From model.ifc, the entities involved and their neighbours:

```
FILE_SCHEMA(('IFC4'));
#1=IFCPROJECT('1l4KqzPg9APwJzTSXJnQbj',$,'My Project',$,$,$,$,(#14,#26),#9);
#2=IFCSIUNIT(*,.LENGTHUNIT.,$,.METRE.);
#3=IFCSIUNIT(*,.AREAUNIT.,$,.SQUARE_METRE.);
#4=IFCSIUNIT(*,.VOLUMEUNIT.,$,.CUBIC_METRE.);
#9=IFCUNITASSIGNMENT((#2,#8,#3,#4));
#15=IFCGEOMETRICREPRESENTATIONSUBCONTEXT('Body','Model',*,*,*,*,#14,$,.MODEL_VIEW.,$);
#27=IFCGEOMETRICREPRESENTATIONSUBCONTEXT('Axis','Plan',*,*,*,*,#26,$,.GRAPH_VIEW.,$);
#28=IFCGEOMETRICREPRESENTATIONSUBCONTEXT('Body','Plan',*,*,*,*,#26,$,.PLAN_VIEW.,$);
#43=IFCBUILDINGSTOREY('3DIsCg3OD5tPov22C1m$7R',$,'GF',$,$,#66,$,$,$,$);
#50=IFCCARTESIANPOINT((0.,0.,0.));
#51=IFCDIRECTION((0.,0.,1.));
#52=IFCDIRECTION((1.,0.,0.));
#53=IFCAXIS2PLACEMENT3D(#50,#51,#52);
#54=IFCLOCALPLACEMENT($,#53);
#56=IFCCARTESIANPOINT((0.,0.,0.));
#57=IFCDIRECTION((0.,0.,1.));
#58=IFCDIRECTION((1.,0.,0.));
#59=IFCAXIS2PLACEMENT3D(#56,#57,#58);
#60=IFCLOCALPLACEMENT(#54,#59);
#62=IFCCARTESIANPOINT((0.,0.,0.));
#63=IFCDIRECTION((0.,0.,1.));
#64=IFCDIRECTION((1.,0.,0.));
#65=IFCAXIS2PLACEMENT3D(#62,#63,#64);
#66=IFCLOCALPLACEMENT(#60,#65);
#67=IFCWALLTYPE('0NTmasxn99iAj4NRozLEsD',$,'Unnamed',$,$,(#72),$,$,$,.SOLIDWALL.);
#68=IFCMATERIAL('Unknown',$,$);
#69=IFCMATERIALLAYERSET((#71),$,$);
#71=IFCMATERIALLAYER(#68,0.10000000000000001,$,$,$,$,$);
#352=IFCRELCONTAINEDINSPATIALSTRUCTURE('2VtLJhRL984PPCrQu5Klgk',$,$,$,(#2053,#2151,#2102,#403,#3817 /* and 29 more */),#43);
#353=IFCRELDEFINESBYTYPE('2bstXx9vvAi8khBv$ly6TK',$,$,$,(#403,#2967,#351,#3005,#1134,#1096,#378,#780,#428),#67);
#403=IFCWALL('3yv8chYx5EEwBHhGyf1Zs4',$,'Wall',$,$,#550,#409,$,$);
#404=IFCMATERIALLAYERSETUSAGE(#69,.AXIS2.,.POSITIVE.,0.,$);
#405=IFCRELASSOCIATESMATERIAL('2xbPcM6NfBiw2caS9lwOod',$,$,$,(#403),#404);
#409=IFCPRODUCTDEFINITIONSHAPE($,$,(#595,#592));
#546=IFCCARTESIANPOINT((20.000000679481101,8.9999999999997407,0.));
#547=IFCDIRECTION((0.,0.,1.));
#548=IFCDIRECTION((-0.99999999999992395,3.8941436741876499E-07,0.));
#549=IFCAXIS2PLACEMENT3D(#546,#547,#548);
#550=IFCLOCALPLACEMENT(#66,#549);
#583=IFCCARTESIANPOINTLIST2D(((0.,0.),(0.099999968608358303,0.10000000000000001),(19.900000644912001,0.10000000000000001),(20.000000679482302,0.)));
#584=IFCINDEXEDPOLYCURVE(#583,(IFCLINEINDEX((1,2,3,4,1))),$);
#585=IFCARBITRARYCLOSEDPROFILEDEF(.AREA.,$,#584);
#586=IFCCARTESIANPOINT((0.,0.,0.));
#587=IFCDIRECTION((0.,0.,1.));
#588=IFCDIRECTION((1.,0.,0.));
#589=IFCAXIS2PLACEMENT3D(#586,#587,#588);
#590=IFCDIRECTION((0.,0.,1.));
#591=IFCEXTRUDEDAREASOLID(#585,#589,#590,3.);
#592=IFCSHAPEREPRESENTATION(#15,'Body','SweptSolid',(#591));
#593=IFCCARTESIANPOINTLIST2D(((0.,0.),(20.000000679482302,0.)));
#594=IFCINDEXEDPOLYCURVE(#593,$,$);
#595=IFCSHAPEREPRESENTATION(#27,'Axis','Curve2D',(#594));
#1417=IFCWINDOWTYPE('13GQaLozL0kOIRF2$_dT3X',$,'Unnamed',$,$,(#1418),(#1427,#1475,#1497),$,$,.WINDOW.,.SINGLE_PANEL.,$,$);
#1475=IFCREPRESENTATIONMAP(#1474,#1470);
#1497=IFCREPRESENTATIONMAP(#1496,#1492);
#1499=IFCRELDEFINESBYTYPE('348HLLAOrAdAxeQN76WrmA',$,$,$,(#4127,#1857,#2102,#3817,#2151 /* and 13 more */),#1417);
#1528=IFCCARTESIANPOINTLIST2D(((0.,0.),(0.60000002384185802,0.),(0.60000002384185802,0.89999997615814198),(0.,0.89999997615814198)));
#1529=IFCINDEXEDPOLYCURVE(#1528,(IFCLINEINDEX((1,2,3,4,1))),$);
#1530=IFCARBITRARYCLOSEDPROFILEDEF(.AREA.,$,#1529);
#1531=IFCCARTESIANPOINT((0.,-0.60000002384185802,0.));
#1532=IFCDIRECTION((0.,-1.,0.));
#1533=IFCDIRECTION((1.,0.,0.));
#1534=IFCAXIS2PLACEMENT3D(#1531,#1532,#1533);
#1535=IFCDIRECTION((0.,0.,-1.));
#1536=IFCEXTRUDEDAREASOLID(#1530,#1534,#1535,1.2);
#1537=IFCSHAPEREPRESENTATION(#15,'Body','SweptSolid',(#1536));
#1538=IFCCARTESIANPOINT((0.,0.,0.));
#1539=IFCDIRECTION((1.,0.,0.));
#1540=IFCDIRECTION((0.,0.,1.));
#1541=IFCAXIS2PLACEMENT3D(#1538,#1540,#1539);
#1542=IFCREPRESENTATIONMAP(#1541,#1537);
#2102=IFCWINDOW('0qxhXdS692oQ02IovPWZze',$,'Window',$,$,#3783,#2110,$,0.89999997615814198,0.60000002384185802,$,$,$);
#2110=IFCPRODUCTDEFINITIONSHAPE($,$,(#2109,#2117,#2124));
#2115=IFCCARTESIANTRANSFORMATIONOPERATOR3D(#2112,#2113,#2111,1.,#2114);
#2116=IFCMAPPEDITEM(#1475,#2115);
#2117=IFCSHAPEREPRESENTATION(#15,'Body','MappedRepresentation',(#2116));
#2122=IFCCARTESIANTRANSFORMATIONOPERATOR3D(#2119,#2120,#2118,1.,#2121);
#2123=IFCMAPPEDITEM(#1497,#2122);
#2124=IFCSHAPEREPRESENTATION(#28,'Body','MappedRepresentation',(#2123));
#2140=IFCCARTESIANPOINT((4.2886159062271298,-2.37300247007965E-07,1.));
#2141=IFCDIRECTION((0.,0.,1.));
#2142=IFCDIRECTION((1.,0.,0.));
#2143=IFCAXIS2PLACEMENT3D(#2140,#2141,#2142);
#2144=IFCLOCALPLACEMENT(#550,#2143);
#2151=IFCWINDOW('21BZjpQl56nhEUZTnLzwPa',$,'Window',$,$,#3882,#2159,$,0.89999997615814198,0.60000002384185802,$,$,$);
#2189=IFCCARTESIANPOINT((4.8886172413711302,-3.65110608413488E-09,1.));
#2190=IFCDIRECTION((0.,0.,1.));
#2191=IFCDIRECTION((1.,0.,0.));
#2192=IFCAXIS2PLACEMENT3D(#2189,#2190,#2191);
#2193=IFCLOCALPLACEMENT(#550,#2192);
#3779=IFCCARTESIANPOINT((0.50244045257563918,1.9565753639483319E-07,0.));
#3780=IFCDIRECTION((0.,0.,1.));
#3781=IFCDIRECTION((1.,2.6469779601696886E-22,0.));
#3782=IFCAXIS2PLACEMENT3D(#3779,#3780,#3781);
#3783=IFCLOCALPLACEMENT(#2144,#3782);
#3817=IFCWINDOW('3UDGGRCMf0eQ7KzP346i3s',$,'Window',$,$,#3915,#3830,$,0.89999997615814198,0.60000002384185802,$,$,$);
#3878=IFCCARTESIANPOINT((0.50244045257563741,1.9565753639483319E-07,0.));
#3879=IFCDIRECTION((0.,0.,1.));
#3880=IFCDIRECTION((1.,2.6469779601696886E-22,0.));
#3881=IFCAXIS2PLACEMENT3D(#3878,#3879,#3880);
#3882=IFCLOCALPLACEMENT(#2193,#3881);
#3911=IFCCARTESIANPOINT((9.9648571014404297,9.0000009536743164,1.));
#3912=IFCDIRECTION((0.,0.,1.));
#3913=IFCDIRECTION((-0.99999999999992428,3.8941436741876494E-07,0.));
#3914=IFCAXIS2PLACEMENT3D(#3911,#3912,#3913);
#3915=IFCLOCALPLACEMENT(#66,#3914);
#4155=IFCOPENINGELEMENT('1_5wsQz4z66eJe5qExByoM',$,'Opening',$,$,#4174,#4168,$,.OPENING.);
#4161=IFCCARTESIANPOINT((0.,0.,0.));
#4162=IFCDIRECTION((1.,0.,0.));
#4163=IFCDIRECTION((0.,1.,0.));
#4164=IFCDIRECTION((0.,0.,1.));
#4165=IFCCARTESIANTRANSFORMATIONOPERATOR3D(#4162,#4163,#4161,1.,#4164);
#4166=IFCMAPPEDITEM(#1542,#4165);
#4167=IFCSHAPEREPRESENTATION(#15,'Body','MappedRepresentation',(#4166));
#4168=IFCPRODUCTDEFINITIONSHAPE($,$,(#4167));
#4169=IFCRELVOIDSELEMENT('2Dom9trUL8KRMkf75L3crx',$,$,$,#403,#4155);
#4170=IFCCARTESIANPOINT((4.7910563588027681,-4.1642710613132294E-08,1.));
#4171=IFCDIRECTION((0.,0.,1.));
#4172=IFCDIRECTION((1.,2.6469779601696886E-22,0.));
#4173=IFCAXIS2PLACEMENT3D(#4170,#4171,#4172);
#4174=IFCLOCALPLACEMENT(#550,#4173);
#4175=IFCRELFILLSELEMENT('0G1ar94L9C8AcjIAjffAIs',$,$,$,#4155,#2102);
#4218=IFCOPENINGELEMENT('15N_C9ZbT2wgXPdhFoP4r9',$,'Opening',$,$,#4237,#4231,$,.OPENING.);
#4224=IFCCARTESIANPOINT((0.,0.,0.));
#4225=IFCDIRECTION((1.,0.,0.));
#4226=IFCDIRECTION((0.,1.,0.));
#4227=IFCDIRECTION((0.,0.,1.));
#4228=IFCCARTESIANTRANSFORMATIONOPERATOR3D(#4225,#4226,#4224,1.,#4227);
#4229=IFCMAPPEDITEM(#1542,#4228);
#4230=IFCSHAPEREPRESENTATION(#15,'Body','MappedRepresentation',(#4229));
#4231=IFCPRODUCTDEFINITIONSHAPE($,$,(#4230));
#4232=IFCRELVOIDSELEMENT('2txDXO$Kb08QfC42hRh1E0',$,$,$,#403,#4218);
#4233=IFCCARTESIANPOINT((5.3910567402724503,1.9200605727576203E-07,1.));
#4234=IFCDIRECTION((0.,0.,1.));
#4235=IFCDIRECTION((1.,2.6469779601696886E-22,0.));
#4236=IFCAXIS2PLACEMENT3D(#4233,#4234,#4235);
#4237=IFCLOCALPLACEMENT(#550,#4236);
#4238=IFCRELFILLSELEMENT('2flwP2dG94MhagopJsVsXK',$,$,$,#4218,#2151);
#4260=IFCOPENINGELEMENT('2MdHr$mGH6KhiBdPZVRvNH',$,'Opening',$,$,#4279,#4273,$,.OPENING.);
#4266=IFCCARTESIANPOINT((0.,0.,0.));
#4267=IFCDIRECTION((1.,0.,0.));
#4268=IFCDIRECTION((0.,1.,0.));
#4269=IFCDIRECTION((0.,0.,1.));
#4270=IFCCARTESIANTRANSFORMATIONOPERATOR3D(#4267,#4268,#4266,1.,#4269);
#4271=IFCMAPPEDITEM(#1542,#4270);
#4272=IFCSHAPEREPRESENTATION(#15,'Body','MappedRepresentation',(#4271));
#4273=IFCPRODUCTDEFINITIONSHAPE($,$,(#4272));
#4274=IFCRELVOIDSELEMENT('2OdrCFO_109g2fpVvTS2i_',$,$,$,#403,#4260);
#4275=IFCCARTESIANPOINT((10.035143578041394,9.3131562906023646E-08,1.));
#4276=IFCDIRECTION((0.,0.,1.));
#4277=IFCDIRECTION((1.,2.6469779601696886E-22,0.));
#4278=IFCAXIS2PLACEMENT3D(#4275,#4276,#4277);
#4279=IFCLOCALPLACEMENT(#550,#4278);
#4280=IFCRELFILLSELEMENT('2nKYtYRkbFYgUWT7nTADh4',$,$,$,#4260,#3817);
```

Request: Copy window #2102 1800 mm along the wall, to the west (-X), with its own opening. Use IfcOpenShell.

```python
import ifcopenshell
import ifcopenshell.api.feature
import ifcopenshell.api.geometry
import ifcopenshell.api.root
import ifcopenshell.geom
import ifcopenshell.util.element
import ifcopenshell.util.placement
import ifcopenshell.util.shape
import ifcopenshell.util.unit

model = ifcopenshell.open("model.ifc")
unit_scale = ifcopenshell.util.unit.calculate_unit_scale(model)
settings = ifcopenshell.geom.settings()


def volume(element):
    """Net volume in cubic metres, openings subtracted."""
    shape = ifcopenshell.geom.create_shape(settings, element)
    return ifcopenshell.util.shape.get_volume(shape.geometry)


window = model.by_guid("0qxhXdS692oQ02IovPWZze")
opening = window.FillsVoids[0].RelatingOpeningElement
wall = opening.VoidsElements[0].RelatingBuildingElement
before = volume(wall)
shift = ifcopenshell.util.placement.get_local_placement(wall.ObjectPlacement)[:3, 0] * 1.8 / unit_scale

# copy_class copies the void relationship, type, container and properties, but no geometry.
new_opening = ifcopenshell.api.root.copy_class(model, product=opening)
new_opening.Representation = ifcopenshell.util.element.copy_deep(
    model, opening.Representation, exclude=["IfcGeometricRepresentationContext", "IfcRepresentationMap"]
)
new_window = ifcopenshell.api.root.copy_class(model, product=window)
new_window.Representation = ifcopenshell.util.element.copy_deep(
    model, window.Representation, exclude=["IfcGeometricRepresentationContext", "IfcRepresentationMap"]
)
ifcopenshell.api.feature.add_filling(model, opening=new_opening, element=new_window)

for old, new in ((opening, new_opening), (window, new_window)):
    matrix = ifcopenshell.util.placement.get_local_placement(old.ObjectPlacement)
    matrix[:3, 3] += shift
    ifcopenshell.api.geometry.edit_object_placement(model, product=new, matrix=matrix, is_si=False)

after = volume(wall)

print(f"wall volume {before:.3f} -> {after:.3f} m3")

model.write("model_edited.ifc")
```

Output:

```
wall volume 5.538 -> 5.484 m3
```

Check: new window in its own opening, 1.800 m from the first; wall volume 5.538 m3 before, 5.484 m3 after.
